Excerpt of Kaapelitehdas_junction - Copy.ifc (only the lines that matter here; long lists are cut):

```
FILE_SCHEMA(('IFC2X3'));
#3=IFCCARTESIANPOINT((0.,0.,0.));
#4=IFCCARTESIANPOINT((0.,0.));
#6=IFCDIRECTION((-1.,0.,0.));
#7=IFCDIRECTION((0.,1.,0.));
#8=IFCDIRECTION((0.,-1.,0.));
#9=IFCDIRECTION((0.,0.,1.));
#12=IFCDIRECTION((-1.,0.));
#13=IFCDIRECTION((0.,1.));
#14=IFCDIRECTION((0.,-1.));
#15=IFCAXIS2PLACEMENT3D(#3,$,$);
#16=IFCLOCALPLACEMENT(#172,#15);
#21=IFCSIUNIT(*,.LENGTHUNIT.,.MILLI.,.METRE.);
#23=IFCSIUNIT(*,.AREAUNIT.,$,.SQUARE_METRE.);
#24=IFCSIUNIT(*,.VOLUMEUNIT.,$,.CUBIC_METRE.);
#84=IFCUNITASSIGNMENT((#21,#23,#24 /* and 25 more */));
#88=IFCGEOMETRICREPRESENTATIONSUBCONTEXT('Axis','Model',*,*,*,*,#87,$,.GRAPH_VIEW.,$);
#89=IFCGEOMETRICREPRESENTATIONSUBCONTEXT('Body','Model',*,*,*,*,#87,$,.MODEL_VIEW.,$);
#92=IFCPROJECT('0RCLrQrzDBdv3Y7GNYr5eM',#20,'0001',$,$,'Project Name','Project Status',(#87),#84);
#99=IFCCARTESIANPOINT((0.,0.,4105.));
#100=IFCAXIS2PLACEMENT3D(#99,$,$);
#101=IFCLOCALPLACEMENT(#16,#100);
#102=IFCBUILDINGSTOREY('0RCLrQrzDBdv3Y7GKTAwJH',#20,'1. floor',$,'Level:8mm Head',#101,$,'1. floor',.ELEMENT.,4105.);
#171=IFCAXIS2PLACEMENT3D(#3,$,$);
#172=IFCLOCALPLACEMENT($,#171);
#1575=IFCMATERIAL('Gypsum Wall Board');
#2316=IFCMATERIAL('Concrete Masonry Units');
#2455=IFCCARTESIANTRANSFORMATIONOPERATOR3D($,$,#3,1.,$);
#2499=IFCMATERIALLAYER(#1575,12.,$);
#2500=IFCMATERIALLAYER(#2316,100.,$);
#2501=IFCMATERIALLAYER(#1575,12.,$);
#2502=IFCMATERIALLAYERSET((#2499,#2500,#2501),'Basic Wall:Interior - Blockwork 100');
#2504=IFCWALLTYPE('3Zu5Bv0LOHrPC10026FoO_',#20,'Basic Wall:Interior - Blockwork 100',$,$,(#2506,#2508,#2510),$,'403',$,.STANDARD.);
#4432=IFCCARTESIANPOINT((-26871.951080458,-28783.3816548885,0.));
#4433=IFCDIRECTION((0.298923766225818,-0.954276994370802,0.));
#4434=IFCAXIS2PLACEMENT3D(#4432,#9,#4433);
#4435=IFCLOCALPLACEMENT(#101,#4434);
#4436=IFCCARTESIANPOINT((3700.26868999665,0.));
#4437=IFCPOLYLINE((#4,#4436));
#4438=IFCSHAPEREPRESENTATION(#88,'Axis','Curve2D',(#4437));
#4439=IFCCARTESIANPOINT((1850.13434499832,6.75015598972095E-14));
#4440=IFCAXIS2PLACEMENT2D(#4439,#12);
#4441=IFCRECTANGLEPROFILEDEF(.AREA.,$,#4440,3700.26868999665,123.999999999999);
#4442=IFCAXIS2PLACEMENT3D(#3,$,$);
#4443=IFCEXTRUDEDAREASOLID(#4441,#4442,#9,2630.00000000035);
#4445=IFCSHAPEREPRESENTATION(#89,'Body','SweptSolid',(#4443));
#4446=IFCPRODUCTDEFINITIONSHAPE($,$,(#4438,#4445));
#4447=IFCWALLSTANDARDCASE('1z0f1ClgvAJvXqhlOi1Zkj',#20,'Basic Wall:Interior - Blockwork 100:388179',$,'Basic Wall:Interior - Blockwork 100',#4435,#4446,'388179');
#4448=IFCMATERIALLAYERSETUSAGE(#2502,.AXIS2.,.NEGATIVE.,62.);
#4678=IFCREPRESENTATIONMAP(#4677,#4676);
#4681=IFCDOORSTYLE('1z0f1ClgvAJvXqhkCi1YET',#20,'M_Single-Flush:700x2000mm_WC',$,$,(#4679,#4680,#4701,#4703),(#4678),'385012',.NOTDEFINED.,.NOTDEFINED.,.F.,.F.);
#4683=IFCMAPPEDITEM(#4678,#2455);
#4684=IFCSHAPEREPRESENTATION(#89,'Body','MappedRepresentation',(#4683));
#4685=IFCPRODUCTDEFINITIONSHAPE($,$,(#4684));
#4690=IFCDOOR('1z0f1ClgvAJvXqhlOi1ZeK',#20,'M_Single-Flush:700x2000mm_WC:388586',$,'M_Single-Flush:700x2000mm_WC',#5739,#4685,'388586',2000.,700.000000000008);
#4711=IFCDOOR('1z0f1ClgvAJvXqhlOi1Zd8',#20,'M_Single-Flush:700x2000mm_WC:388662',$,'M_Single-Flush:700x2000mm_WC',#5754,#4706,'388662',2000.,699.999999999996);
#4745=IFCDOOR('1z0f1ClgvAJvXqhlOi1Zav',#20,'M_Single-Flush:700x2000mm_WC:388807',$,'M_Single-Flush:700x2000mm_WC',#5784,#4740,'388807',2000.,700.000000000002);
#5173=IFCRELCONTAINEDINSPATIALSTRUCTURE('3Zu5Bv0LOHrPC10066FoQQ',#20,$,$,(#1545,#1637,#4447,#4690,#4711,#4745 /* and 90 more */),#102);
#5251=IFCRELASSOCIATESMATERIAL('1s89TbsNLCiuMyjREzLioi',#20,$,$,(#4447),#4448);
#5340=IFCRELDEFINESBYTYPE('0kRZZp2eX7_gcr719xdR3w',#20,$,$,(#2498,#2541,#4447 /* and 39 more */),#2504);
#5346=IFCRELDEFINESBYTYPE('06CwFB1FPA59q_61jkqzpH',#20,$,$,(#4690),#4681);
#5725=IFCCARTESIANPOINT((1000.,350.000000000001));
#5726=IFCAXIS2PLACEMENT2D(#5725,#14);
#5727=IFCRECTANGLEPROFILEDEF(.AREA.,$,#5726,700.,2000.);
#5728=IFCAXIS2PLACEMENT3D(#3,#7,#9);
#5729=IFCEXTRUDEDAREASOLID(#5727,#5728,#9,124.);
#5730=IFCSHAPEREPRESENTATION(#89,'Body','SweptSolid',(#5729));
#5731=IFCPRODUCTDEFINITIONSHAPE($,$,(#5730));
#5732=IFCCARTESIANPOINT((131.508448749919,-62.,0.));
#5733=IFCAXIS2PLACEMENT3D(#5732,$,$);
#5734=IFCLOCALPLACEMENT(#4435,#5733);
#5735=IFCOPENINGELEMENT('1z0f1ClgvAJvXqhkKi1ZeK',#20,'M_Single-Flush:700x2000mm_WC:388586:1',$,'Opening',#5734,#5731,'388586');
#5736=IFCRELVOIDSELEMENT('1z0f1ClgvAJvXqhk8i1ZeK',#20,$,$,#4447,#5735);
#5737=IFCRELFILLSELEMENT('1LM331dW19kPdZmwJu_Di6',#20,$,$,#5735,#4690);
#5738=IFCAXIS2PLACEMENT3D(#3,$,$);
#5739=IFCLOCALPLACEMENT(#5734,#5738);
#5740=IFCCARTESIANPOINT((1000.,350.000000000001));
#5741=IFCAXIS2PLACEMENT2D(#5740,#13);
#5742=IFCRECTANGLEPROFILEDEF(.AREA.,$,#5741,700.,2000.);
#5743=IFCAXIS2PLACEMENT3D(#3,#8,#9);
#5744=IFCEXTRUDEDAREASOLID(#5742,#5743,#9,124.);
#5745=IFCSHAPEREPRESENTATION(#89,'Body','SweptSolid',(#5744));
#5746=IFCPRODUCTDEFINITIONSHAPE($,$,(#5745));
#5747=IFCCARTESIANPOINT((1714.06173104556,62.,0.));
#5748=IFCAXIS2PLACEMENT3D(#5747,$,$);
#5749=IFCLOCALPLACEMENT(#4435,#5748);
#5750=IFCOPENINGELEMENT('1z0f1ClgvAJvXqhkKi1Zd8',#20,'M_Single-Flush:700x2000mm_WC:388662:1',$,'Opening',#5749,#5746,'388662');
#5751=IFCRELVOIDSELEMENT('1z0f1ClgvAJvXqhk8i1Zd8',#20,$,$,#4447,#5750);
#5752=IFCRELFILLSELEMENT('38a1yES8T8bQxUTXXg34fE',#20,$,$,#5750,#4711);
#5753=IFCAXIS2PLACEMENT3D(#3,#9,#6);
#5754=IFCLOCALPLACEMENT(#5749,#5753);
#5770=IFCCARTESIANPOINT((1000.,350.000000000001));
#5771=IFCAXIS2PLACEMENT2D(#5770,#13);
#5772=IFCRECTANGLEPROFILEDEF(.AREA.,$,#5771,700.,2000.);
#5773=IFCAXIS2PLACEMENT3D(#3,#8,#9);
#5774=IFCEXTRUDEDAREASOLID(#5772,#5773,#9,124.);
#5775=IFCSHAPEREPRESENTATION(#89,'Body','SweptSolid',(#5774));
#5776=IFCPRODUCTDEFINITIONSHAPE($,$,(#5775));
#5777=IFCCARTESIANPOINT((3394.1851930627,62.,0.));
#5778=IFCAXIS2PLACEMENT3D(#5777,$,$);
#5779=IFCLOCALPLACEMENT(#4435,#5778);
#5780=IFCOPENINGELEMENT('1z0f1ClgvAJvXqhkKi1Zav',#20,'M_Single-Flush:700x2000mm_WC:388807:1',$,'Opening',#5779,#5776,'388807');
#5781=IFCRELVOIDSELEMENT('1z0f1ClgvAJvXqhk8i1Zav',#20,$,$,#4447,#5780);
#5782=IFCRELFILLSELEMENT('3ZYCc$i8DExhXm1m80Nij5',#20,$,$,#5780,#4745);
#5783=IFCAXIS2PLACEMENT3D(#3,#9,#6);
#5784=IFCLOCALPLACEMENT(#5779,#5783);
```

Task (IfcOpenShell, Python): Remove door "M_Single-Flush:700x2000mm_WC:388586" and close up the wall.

```python
import ifcopenshell
import ifcopenshell.api.feature
import ifcopenshell.api.root
import ifcopenshell.geom
import ifcopenshell.util.shape

model = ifcopenshell.open("Kaapelitehdas_junction - Copy.ifc")
settings = ifcopenshell.geom.settings()


def volume(element):
    """Net volume in cubic metres, openings subtracted."""
    shape = ifcopenshell.geom.create_shape(settings, element)
    return ifcopenshell.util.shape.get_volume(shape.geometry)


door = model.by_id(4690)
opening = door.FillsVoids[0].RelatingOpeningElement
wall = opening.VoidsElements[0].RelatingBuildingElement
before = volume(wall)

ifcopenshell.api.root.remove_product(model, product=door)
ifcopenshell.api.feature.remove_feature(model, feature=opening)

after = volume(wall)

print(f"wall volume {before:.3f} -> {after:.3f} m3")

model.write("Kaapelitehdas_junction - Copy_rev.ifc")
```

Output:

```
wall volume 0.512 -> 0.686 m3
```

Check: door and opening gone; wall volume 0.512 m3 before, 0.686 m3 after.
